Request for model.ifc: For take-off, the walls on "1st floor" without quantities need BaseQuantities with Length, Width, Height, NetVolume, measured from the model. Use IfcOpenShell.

First a look at what the model holds.

```python
import ifcopenshell
import ifcopenshell.util.element
import ifcopenshell.util.unit

model = ifcopenshell.open("model.ifc")
print(model.schema)
for unit_type in ("LENGTHUNIT", "AREAUNIT", "VOLUMEUNIT"):
    print(unit_type, ifcopenshell.util.unit.calculate_unit_scale(model, unit_type))
storey = next(s for s in model.by_type("IfcBuildingStorey") if s.Name == "1st floor")
walls = [e for e in ifcopenshell.util.element.get_decomposition(storey) if e.is_a("IfcWall")]
for e in sorted(walls, key=lambda e: e.id()):
    print(e.id(), e.is_a(), e.Name, list(ifcopenshell.util.element.get_psets(e, qtos_only=True)), sep=" | ")
```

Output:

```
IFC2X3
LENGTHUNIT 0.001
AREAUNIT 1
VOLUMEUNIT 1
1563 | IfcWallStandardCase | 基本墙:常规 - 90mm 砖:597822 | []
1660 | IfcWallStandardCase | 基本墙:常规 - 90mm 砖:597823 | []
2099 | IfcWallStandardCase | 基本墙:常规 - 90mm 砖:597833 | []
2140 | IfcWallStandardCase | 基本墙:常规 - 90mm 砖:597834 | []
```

```python
import ifcopenshell
import ifcopenshell.api.pset
import ifcopenshell.geom
import ifcopenshell.util.element
import ifcopenshell.util.shape
import ifcopenshell.util.unit

model = ifcopenshell.open("model.ifc")
unit_scale = ifcopenshell.util.unit.calculate_unit_scale(model)
volume_scale = ifcopenshell.util.unit.calculate_unit_scale(model, "VOLUMEUNIT")
settings = ifcopenshell.geom.settings()

storey = next(s for s in model.by_type("IfcBuildingStorey") if s.Name == "1st floor")
walls = [e for e in ifcopenshell.util.element.get_decomposition(storey) if e.is_a("IfcWall")]

for e in sorted(walls, key=lambda e: e.id()):
    if ifcopenshell.util.element.get_psets(e, qtos_only=True, should_inherit=False):
        continue
    # Geometry comes back in metres, in the element's own axes.
    shape = ifcopenshell.geom.create_shape(settings, e)
    values = {
        "Length": ifcopenshell.util.shape.get_x(shape.geometry) / unit_scale,
        "Width": ifcopenshell.util.shape.get_y(shape.geometry) / unit_scale,
        "Height": ifcopenshell.util.shape.get_z(shape.geometry) / unit_scale,
        "NetVolume": ifcopenshell.util.shape.get_volume(shape.geometry) / volume_scale,
    }
    qto = ifcopenshell.api.pset.add_qto(model, product=e, name="BaseQuantities")
    ifcopenshell.api.pset.edit_qto(model, qto=qto, properties=values)
    print(e.id(), {k: round(v, 3) for k, v in values.items()})

model.write("model_updated.ifc")
```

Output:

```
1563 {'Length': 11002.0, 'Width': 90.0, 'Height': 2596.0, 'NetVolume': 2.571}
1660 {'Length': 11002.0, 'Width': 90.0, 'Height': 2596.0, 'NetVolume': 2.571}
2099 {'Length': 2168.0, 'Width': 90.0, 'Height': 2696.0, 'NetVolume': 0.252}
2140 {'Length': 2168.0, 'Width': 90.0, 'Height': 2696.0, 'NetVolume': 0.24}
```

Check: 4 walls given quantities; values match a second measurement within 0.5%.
